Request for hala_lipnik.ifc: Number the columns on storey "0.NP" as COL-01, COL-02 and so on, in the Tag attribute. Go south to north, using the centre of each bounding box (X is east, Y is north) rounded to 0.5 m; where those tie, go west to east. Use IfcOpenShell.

First a look at what the model holds.

```python
import ifcopenshell
import ifcopenshell.util.element
import ifcopenshell.util.placement

model = ifcopenshell.open("hala_lipnik.ifc")
print(model.schema)
storey = next(s for s in model.by_type("IfcBuildingStorey") if s.Name == "0.NP")
columns = [e for e in ifcopenshell.util.element.get_decomposition(storey) if e.is_a("IfcColumn")]
for e in sorted(columns, key=lambda e: e.id()):
    origin = ifcopenshell.util.placement.get_local_placement(e.ObjectPlacement)[:3, 3]
    print(e.id(), e.Tag, e.Name, origin.round(2) + 0.0, sep=" | ")
```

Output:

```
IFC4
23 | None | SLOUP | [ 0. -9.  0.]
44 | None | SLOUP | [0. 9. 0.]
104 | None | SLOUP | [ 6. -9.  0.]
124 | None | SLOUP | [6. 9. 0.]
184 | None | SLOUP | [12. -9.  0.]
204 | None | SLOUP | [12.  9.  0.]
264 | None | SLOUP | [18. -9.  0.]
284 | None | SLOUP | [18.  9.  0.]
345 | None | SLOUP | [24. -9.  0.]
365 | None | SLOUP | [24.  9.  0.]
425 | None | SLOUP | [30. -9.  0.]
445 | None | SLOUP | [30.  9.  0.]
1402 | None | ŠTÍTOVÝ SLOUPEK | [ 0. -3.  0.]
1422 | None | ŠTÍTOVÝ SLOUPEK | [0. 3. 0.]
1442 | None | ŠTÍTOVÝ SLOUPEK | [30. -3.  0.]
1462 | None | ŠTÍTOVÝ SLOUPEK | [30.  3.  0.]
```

```python
import ifcopenshell
import ifcopenshell.geom
import ifcopenshell.util.element
import ifcopenshell.util.shape

model = ifcopenshell.open("hala_lipnik.ifc")
settings = ifcopenshell.geom.settings()
settings.set("use-world-coords", True)


def centre(element):
    shape = ifcopenshell.geom.create_shape(settings, element)
    return ifcopenshell.util.shape.get_bbox_centroid(shape.geometry)


storey = next(s for s in model.by_type("IfcBuildingStorey") if s.Name == "0.NP")
columns = [e for e in ifcopenshell.util.element.get_decomposition(storey) if e.is_a("IfcColumn")]

# Insertion points can sit at a corner or the storey origin, so sort by the geometry (in metres).
centres = {e: centre(e) for e in columns}
columns.sort(key=lambda e: (round(centres[e][1] / 0.5), centres[e][0]))

for i, e in enumerate(columns, start=1):
    number = f"COL-{i:02d}"
    e.Tag = number
    print(e.id(), number)

model.write("hala_lipnik_edited.ifc")
```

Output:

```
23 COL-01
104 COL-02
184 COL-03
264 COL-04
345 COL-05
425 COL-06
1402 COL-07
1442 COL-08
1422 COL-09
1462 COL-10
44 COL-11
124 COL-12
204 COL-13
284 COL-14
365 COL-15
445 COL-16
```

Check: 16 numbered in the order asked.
